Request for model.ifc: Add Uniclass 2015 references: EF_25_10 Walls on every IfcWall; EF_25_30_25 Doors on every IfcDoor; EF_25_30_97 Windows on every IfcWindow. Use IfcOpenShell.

First a look at what the model holds.

```python
import ifcopenshell

model = ifcopenshell.open("model.ifc")
print(model.schema)
print("classifications:", [c.Name for c in model.by_type("IfcClassification")])
for ifc_class in ("IfcDoor", "IfcRoof", "IfcStair", "IfcWall", "IfcWindow"):
    print(ifc_class, len(model.by_type(ifc_class)))
```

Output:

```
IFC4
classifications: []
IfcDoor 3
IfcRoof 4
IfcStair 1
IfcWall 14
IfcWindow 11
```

```python
import ifcopenshell
import ifcopenshell.api.classification

model = ifcopenshell.open("model.ifc")

system = ifcopenshell.api.classification.add_classification(model, classification="Uniclass 2015")

codes = {
    "IfcWall": ("EF_25_10", "Walls"),
    "IfcDoor": ("EF_25_30_25", "Doors"),
    "IfcWindow": ("EF_25_30_97", "Windows"),
}
for ifc_class, (code, name) in codes.items():
    products = model.by_type(ifc_class)
    ifcopenshell.api.classification.add_reference(
        model, products=products, classification=system, identification=code, name=name
    )
    print(code, len(products))

model.write("model_rev.ifc")
```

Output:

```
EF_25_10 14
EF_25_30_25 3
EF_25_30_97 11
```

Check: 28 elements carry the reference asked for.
